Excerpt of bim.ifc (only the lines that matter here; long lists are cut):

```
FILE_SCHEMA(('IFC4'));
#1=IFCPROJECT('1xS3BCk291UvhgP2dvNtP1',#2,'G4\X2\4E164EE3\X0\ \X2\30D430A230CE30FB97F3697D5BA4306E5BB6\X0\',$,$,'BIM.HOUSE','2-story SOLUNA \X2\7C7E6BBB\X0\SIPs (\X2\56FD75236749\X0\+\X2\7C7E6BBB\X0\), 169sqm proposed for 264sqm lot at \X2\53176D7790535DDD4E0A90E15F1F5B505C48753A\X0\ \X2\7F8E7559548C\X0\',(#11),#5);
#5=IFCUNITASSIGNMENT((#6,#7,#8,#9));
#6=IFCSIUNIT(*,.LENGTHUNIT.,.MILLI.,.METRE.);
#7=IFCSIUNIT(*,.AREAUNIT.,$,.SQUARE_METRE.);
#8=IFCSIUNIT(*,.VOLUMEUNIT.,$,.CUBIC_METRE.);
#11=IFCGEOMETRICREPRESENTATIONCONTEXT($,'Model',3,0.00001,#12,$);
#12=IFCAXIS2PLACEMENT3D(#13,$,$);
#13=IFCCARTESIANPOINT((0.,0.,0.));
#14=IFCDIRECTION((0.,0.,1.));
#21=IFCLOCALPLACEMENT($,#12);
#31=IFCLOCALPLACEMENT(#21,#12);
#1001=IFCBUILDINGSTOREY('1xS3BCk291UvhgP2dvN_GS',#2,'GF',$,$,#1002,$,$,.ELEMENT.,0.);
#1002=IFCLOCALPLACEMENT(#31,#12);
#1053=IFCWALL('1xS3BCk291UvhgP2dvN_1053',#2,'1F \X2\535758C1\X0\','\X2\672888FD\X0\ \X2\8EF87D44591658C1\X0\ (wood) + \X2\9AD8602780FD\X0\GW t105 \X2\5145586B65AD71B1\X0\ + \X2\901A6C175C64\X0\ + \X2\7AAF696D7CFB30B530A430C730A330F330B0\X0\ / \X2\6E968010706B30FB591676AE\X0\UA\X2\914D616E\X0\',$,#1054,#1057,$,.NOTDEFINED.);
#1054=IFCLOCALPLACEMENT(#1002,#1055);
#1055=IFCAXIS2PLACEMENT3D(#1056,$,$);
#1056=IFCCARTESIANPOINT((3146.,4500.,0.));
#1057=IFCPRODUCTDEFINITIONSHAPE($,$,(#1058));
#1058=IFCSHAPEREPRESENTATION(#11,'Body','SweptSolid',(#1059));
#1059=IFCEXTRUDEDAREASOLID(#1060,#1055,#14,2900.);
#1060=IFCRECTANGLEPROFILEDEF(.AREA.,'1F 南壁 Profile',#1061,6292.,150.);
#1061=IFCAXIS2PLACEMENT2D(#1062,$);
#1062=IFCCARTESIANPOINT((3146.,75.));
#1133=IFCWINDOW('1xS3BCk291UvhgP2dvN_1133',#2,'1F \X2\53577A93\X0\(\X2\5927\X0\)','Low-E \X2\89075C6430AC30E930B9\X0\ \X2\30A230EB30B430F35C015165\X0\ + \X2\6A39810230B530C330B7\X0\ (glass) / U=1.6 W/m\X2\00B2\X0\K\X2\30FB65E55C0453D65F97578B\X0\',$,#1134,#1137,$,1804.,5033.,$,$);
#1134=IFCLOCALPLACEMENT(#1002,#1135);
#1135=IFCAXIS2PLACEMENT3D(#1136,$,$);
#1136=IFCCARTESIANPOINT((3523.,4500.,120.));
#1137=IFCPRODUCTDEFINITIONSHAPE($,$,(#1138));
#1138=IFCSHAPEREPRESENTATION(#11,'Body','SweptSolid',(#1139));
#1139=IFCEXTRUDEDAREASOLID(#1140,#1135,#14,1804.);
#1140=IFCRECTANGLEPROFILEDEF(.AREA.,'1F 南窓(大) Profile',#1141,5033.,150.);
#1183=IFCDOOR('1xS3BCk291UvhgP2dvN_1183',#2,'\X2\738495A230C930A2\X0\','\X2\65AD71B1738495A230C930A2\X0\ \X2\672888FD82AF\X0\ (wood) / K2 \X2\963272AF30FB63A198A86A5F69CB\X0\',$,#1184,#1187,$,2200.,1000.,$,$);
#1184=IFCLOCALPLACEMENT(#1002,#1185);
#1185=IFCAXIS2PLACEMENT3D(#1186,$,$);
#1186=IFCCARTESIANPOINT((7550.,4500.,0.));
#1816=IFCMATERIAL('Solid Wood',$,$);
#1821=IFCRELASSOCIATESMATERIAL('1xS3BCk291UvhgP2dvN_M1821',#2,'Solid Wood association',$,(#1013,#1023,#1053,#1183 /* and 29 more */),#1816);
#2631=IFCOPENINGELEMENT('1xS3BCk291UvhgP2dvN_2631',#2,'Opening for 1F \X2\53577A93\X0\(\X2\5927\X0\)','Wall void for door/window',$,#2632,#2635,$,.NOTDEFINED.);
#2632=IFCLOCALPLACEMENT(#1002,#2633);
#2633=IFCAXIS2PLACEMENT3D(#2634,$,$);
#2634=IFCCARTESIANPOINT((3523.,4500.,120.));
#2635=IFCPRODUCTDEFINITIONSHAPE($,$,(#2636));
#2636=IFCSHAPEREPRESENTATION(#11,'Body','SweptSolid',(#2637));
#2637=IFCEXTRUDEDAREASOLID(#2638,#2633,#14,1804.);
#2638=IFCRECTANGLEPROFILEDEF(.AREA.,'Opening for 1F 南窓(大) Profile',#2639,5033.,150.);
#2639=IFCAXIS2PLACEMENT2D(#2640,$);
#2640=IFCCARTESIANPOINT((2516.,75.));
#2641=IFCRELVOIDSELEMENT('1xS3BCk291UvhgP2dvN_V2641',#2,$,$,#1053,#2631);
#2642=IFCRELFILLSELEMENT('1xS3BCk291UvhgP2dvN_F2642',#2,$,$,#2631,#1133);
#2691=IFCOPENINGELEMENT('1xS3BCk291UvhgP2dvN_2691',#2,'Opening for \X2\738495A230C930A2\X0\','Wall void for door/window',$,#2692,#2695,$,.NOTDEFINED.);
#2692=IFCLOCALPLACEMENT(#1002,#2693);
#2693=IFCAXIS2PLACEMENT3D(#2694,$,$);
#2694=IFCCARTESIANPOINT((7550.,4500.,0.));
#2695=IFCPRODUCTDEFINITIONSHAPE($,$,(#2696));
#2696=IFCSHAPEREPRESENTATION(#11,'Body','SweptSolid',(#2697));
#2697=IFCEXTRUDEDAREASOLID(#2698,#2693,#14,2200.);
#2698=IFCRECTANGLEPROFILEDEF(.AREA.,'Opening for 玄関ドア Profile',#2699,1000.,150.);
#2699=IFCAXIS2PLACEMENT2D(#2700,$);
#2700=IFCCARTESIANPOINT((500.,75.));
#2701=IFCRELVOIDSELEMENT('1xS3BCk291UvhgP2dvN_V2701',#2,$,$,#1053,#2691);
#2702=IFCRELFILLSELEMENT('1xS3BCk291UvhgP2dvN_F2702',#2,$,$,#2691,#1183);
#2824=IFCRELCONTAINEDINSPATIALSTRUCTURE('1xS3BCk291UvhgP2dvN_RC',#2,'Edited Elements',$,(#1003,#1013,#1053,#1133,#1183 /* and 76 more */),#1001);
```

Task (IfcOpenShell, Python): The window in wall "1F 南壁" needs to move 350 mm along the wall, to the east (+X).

```python
import ifcopenshell
import ifcopenshell.api.geometry
import ifcopenshell.util.placement
import ifcopenshell.util.unit

model = ifcopenshell.open("bim.ifc")
unit_scale = ifcopenshell.util.unit.calculate_unit_scale(model)

window = model.by_id(1133)
opening = window.FillsVoids[0].RelatingOpeningElement
wall = opening.VoidsElements[0].RelatingBuildingElement

wall_matrix = ifcopenshell.util.placement.get_local_placement(wall.ObjectPlacement)
shift = wall_matrix[:3, 0] * 0.35 / unit_scale
before = ifcopenshell.util.placement.get_local_placement(window.ObjectPlacement)[:3, 3].copy()

# The window is not placed relative to its opening, so move both.
for product in (opening, window):
    matrix = ifcopenshell.util.placement.get_local_placement(product.ObjectPlacement)
    matrix[:3, 3] += shift
    ifcopenshell.api.geometry.edit_object_placement(model, product=product, matrix=matrix, is_si=False)

after = ifcopenshell.util.placement.get_local_placement(window.ObjectPlacement)[:3, 3]
print("window moved by", (after - before).round(3) + 0.0)

model.write("bim_edited.ifc")
```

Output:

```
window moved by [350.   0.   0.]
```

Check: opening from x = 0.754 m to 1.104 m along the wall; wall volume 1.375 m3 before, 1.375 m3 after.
